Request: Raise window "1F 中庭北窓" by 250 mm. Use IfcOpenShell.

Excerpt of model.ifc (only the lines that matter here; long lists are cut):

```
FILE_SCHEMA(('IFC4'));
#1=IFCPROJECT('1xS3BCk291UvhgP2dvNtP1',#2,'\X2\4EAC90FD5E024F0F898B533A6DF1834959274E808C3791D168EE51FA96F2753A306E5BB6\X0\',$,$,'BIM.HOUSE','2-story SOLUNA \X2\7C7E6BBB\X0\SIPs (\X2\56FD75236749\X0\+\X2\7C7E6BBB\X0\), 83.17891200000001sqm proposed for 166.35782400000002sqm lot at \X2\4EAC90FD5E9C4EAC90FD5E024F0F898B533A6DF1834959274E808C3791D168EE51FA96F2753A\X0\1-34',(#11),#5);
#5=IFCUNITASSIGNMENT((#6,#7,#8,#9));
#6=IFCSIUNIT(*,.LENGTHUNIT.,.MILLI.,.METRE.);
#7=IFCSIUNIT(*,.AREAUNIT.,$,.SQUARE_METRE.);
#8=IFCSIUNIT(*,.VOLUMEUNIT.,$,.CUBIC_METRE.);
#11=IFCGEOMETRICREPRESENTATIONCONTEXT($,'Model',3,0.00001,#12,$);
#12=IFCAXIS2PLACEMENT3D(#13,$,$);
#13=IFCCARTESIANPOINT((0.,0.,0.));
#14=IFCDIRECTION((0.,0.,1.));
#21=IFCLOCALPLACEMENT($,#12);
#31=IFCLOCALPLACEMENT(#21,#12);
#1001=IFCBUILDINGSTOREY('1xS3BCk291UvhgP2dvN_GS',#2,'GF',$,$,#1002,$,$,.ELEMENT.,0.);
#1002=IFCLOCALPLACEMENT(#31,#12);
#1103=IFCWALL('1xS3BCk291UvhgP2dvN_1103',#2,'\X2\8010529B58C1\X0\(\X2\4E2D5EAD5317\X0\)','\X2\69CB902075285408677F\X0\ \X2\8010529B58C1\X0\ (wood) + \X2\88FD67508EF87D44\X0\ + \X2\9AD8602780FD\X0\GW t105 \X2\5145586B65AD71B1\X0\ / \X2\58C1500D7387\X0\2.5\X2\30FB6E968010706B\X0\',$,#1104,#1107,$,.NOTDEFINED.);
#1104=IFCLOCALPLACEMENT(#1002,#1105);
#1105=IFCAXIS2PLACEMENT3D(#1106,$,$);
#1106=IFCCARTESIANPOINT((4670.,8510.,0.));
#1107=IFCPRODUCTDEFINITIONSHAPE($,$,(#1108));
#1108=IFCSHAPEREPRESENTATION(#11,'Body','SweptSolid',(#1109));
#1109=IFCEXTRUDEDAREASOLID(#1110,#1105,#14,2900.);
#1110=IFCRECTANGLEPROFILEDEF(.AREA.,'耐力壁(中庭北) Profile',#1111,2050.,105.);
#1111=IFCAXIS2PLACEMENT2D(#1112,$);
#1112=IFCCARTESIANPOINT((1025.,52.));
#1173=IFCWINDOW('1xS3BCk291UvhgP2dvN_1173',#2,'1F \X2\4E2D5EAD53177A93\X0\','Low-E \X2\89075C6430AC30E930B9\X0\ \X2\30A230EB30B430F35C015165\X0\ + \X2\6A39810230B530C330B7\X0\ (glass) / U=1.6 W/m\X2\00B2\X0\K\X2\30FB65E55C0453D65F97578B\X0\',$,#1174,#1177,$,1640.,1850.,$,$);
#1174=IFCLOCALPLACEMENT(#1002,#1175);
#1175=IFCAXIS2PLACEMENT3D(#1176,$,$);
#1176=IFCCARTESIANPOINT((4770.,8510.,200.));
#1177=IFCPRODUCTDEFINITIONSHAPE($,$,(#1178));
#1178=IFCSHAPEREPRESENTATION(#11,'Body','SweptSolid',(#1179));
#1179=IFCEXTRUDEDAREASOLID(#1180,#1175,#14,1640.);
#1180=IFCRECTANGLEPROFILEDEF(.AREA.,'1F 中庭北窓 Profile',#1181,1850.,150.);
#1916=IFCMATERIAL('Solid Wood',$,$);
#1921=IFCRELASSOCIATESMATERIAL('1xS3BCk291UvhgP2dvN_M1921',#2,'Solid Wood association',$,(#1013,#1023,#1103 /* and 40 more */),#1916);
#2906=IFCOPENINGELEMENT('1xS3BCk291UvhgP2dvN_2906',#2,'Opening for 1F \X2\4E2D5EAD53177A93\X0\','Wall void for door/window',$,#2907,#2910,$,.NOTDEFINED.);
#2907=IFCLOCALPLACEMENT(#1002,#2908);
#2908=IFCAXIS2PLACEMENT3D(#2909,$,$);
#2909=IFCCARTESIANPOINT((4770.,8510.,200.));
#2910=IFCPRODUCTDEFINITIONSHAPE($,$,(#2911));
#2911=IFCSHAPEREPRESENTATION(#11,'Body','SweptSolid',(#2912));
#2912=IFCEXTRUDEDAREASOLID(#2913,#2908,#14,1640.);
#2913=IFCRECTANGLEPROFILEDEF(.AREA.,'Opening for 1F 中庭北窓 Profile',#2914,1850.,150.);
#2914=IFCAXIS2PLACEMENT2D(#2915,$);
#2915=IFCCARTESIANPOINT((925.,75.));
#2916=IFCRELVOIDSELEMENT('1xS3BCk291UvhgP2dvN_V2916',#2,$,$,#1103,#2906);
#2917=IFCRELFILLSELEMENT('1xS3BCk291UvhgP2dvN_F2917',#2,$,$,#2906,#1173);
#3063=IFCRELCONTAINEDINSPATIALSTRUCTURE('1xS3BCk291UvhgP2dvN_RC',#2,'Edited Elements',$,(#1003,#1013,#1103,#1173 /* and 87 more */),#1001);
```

```python
import numpy as np
import ifcopenshell
import ifcopenshell.api.geometry
import ifcopenshell.util.placement
import ifcopenshell.util.unit

model = ifcopenshell.open("model.ifc")
unit_scale = ifcopenshell.util.unit.calculate_unit_scale(model)

window = model.by_guid("1xS3BCk291UvhgP2dvN_1173")
opening = window.FillsVoids[0].RelatingOpeningElement
dz = 0.25 / unit_scale

shift = np.array([0.0, 0.0, dz])
# The window is not placed relative to its opening, so move both.
for product in (opening, window):
    matrix = ifcopenshell.util.placement.get_local_placement(product.ObjectPlacement)
    matrix[:3, 3] += shift
    ifcopenshell.api.geometry.edit_object_placement(model, product=product, matrix=matrix, is_si=False)

print(f"moved by {dz * unit_scale:+.3f} m")

model.write("model-out.ifc")
```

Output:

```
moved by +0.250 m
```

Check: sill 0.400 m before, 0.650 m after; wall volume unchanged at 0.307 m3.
